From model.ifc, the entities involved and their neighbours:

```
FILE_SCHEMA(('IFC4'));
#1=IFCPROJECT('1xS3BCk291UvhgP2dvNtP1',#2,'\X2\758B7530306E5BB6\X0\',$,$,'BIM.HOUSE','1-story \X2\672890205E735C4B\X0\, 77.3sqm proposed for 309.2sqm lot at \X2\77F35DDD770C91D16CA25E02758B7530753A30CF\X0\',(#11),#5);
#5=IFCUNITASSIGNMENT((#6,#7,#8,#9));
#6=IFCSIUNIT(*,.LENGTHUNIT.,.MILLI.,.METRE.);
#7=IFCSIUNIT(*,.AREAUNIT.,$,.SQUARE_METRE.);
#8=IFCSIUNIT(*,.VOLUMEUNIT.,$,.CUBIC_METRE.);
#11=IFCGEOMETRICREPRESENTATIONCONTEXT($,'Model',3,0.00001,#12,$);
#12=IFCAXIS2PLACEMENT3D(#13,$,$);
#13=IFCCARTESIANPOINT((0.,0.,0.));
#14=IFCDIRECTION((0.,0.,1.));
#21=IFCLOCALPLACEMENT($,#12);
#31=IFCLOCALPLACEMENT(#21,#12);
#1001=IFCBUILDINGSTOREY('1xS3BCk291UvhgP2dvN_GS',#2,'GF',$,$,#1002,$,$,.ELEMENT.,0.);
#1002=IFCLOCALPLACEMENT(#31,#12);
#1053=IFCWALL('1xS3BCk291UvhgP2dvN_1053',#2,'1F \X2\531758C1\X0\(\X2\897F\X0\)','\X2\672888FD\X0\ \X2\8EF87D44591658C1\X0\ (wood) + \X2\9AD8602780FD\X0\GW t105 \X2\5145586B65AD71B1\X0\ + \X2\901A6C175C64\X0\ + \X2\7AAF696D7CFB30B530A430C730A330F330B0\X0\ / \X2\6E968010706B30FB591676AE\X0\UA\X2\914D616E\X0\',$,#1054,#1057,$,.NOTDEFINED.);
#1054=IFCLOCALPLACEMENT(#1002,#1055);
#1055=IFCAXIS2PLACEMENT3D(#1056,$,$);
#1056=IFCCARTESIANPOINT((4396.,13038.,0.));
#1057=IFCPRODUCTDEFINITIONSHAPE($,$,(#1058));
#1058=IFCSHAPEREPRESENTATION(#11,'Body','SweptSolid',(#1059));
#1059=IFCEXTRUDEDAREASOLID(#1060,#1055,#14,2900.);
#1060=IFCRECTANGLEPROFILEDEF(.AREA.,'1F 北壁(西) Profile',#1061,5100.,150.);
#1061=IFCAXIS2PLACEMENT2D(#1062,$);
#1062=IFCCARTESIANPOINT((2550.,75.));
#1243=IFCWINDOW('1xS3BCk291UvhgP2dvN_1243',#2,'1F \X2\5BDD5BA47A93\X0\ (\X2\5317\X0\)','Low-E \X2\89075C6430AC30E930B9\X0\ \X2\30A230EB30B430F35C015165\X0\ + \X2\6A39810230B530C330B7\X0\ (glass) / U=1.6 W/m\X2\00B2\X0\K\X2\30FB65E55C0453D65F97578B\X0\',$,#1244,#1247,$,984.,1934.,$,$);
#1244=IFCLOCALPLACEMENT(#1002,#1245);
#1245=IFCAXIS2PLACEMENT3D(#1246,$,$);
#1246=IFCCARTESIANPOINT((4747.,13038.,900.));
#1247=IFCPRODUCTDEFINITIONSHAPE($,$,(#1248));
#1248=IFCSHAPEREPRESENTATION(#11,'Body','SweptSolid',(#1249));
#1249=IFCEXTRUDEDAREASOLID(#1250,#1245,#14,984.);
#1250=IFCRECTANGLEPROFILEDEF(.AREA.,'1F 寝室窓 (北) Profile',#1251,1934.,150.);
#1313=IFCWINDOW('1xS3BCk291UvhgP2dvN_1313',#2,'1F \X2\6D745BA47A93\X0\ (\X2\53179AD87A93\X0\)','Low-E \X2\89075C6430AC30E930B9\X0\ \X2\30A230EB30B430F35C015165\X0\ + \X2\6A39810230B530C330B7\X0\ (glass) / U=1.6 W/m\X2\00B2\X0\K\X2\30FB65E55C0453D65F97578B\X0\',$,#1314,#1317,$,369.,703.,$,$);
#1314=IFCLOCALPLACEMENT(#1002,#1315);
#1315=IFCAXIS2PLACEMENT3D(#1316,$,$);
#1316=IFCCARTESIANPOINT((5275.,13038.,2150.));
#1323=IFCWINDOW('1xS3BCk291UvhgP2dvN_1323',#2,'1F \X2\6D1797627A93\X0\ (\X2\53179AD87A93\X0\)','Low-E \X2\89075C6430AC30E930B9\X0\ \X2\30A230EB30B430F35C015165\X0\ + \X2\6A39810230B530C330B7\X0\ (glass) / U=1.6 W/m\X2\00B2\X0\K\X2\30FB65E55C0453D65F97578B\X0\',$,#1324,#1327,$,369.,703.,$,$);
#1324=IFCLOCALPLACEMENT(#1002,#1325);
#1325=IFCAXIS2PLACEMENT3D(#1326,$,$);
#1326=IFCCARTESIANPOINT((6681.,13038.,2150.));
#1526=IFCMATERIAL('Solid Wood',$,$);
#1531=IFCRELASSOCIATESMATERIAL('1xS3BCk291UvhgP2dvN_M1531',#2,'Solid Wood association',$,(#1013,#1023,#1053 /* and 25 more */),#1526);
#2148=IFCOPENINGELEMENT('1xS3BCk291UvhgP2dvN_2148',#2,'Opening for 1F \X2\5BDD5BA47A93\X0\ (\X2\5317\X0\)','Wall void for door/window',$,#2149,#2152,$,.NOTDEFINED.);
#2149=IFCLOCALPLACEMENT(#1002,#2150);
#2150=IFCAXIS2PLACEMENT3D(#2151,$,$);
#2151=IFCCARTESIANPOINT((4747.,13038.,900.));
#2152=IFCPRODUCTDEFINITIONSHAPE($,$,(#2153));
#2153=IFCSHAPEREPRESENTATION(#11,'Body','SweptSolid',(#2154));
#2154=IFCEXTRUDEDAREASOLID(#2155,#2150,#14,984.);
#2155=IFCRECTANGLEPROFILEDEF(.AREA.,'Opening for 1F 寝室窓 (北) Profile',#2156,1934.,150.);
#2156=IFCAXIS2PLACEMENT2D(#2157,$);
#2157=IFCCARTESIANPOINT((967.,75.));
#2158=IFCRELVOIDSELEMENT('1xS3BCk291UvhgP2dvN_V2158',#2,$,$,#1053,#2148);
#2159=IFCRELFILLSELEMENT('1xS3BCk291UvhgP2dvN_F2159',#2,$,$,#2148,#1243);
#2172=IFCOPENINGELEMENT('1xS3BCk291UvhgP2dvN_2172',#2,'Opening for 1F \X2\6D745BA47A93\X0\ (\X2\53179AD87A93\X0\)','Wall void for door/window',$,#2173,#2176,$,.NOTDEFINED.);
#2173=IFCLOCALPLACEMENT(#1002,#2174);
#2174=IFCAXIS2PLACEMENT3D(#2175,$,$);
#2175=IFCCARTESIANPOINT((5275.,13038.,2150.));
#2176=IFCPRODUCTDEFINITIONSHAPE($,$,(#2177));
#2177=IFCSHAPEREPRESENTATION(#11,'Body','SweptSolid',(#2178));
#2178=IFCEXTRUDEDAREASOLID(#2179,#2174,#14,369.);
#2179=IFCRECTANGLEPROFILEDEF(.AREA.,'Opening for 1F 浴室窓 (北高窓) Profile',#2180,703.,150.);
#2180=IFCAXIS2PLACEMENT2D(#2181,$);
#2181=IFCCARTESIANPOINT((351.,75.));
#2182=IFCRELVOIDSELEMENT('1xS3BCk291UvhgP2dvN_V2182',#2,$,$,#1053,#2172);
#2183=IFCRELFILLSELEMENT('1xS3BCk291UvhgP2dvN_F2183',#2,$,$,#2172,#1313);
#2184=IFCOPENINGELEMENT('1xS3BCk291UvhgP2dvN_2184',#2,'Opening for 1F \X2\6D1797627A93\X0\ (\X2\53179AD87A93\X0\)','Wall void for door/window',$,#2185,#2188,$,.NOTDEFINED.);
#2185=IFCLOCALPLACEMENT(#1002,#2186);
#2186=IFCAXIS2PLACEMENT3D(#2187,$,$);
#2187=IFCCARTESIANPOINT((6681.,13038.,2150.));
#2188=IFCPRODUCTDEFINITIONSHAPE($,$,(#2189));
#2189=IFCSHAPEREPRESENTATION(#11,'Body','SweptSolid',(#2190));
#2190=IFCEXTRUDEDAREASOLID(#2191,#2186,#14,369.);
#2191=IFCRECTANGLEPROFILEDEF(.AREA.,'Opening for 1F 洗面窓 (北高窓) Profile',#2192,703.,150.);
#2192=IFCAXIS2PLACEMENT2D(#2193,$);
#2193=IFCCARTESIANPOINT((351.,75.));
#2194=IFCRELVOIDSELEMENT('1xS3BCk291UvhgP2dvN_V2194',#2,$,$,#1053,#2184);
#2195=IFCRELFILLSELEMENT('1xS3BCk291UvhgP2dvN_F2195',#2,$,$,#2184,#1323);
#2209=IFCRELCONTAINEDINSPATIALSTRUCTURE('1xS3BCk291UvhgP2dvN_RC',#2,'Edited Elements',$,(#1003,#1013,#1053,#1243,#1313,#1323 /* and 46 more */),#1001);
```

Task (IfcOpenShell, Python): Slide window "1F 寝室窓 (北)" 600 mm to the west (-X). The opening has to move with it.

```python
import ifcopenshell
import ifcopenshell.api.geometry
import ifcopenshell.util.placement

model = ifcopenshell.open("model.ifc")

window = model.by_guid("1xS3BCk291UvhgP2dvN_1243")
opening = window.FillsVoids[0].RelatingOpeningElement
wall = opening.VoidsElements[0].RelatingBuildingElement

wall_matrix = ifcopenshell.util.placement.get_local_placement(wall.ObjectPlacement)
shift = wall_matrix[:3, 0] * -600.0
before = ifcopenshell.util.placement.get_local_placement(window.ObjectPlacement)[:3, 3].copy()

# The window is not placed relative to its opening, so move both.
for product in (opening, window):
    matrix = ifcopenshell.util.placement.get_local_placement(product.ObjectPlacement)
    matrix[:3, 3] += shift
    ifcopenshell.api.geometry.edit_object_placement(model, product=product, matrix=matrix, is_si=False)

after = ifcopenshell.util.placement.get_local_placement(window.ObjectPlacement)[:3, 3]
print("window moved by", (after - before).round(3) + 0.0)

model.write("model_updated.ifc")
```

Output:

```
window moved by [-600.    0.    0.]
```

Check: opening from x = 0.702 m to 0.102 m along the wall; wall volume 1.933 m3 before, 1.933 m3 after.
